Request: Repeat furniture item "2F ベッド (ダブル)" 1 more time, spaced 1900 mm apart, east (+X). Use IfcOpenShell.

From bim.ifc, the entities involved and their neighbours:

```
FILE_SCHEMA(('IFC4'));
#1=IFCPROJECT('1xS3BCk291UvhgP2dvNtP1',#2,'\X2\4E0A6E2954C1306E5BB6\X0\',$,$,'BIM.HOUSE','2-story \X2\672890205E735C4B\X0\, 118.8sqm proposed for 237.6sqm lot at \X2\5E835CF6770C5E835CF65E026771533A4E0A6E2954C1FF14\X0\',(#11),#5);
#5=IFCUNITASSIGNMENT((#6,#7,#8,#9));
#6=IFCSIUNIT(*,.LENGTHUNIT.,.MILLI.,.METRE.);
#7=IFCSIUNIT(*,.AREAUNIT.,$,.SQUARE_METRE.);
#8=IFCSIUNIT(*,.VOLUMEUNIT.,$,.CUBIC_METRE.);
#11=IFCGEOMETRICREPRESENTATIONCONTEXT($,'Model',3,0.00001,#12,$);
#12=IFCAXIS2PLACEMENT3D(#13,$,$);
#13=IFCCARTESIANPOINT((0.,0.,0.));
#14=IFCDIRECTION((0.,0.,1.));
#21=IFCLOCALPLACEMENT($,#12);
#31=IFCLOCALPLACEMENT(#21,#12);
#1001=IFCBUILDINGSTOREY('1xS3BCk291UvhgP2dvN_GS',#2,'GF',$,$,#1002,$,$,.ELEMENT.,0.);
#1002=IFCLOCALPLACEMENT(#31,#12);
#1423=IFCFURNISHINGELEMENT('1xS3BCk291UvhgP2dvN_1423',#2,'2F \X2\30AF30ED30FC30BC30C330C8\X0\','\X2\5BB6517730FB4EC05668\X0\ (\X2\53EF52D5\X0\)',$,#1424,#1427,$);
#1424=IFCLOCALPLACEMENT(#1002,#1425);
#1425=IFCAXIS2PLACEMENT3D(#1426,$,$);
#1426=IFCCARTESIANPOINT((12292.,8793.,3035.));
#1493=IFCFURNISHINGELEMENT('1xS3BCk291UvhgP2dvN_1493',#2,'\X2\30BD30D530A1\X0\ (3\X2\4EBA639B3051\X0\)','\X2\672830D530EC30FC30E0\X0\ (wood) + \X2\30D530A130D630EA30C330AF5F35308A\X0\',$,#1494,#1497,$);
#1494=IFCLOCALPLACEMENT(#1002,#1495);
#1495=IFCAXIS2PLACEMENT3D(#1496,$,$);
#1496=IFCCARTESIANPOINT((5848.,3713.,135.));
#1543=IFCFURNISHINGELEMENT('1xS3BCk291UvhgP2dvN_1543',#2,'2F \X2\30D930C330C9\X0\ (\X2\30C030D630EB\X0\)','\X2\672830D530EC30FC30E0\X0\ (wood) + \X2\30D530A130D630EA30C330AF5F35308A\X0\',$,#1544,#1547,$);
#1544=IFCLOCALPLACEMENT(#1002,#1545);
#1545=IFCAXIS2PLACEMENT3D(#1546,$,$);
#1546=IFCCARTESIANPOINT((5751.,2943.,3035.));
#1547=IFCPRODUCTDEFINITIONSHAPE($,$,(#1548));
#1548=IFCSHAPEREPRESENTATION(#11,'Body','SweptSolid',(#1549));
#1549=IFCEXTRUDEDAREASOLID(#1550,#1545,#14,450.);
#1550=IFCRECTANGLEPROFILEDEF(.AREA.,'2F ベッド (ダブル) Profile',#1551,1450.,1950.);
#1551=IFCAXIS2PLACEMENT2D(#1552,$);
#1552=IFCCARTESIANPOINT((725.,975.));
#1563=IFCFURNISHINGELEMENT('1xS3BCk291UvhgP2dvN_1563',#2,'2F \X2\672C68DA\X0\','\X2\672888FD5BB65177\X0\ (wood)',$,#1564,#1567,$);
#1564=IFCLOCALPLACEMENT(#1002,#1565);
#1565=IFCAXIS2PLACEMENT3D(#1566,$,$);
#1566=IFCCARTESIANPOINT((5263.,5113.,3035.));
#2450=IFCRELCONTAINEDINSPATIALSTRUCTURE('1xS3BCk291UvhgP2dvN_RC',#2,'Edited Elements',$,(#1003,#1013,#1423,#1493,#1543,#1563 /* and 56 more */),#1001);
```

```python
import numpy as np
import ifcopenshell
import ifcopenshell.api.geometry
import ifcopenshell.api.root
import ifcopenshell.util.element
import ifcopenshell.util.placement
import ifcopenshell.util.unit

model = ifcopenshell.open("bim.ifc")
unit_scale = ifcopenshell.util.unit.calculate_unit_scale(model)


def reuse_history(source, copy):
    """copy_class also copies each property set's owner history, people and application; keep the originals."""
    for rel in copy.IsDefinedBy:
        if rel.is_a("IfcRelDefinesByProperties") and (history := rel.RelatingPropertyDefinition.OwnerHistory):
            rel.RelatingPropertyDefinition.OwnerHistory = source.OwnerHistory
            ifcopenshell.util.element.remove_deep2(model, history)


source = model.by_guid("1xS3BCk291UvhgP2dvN_1543")
base = ifcopenshell.util.placement.get_local_placement(source.ObjectPlacement)
step = np.array([1.0, 0.0, 0.0]) * 1.9 / unit_scale

for i in range(1, 2):
    copy = ifcopenshell.api.root.copy_class(model, product=source)
    copy.Representation = ifcopenshell.util.element.copy_deep(
        model, source.Representation, exclude=["IfcGeometricRepresentationContext", "IfcRepresentationMap"]
    )
    reuse_history(source, copy)
    matrix = base.copy()
    matrix[:3, 3] += i * step
    print("added at", matrix[:3, 3].round(3) + 0.0)
    ifcopenshell.api.geometry.edit_object_placement(model, product=copy, matrix=matrix, is_si=False)

model.write("bim_updated.ifc")
```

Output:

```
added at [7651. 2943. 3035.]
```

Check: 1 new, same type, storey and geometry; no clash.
